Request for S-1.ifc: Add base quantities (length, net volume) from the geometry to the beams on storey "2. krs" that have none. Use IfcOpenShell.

First a look at what the model holds.

```python
import ifcopenshell
import ifcopenshell.util.element
import ifcopenshell.util.unit

model = ifcopenshell.open("S-1.ifc")
print(model.schema)
for unit_type in ("LENGTHUNIT", "AREAUNIT", "VOLUMEUNIT"):
    print(unit_type, ifcopenshell.util.unit.calculate_unit_scale(model, unit_type))
storey = next(s for s in model.by_type("IfcBuildingStorey") if s.Name == "2. krs")
beams = [e for e in ifcopenshell.util.element.get_decomposition(storey) if e.is_a("IfcBeam")]
for e in sorted(beams, key=lambda e: e.id()):
    print(e.id(), e.is_a(), e.Name, list(ifcopenshell.util.element.get_psets(e, qtos_only=True)), sep=" | ")
```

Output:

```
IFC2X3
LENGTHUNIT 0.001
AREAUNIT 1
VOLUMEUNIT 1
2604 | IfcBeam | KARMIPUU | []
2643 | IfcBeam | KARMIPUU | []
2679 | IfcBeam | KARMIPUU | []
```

```python
import ifcopenshell
import ifcopenshell.api.pset
import ifcopenshell.geom
import ifcopenshell.util.element
import ifcopenshell.util.shape
import ifcopenshell.util.unit

model = ifcopenshell.open("S-1.ifc")
unit_scale = ifcopenshell.util.unit.calculate_unit_scale(model)
volume_scale = ifcopenshell.util.unit.calculate_unit_scale(model, "VOLUMEUNIT")
settings = ifcopenshell.geom.settings()

storey = next(s for s in model.by_type("IfcBuildingStorey") if s.Name == "2. krs")
beams = [e for e in ifcopenshell.util.element.get_decomposition(storey) if e.is_a("IfcBeam")]

for e in sorted(beams, key=lambda e: e.id()):
    if ifcopenshell.util.element.get_psets(e, qtos_only=True, should_inherit=False):
        continue
    # Geometry comes back in metres, in the element's own axes.
    shape = ifcopenshell.geom.create_shape(settings, e)
    values = {
        "Length": ifcopenshell.util.shape.get_max_xyz(shape.geometry) / unit_scale,
        "NetVolume": ifcopenshell.util.shape.get_volume(shape.geometry) / volume_scale,
    }
    qto = ifcopenshell.api.pset.add_qto(model, product=e, name="BaseQuantities")
    ifcopenshell.api.pset.edit_qto(model, qto=qto, properties=values)
    print(e.id(), {k: round(v, 3) for k, v in values.items()})

model.write("S-1_updated.ifc")
```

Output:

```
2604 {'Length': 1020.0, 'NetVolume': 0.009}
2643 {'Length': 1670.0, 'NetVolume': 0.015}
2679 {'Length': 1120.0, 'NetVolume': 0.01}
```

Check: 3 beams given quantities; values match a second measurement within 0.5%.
